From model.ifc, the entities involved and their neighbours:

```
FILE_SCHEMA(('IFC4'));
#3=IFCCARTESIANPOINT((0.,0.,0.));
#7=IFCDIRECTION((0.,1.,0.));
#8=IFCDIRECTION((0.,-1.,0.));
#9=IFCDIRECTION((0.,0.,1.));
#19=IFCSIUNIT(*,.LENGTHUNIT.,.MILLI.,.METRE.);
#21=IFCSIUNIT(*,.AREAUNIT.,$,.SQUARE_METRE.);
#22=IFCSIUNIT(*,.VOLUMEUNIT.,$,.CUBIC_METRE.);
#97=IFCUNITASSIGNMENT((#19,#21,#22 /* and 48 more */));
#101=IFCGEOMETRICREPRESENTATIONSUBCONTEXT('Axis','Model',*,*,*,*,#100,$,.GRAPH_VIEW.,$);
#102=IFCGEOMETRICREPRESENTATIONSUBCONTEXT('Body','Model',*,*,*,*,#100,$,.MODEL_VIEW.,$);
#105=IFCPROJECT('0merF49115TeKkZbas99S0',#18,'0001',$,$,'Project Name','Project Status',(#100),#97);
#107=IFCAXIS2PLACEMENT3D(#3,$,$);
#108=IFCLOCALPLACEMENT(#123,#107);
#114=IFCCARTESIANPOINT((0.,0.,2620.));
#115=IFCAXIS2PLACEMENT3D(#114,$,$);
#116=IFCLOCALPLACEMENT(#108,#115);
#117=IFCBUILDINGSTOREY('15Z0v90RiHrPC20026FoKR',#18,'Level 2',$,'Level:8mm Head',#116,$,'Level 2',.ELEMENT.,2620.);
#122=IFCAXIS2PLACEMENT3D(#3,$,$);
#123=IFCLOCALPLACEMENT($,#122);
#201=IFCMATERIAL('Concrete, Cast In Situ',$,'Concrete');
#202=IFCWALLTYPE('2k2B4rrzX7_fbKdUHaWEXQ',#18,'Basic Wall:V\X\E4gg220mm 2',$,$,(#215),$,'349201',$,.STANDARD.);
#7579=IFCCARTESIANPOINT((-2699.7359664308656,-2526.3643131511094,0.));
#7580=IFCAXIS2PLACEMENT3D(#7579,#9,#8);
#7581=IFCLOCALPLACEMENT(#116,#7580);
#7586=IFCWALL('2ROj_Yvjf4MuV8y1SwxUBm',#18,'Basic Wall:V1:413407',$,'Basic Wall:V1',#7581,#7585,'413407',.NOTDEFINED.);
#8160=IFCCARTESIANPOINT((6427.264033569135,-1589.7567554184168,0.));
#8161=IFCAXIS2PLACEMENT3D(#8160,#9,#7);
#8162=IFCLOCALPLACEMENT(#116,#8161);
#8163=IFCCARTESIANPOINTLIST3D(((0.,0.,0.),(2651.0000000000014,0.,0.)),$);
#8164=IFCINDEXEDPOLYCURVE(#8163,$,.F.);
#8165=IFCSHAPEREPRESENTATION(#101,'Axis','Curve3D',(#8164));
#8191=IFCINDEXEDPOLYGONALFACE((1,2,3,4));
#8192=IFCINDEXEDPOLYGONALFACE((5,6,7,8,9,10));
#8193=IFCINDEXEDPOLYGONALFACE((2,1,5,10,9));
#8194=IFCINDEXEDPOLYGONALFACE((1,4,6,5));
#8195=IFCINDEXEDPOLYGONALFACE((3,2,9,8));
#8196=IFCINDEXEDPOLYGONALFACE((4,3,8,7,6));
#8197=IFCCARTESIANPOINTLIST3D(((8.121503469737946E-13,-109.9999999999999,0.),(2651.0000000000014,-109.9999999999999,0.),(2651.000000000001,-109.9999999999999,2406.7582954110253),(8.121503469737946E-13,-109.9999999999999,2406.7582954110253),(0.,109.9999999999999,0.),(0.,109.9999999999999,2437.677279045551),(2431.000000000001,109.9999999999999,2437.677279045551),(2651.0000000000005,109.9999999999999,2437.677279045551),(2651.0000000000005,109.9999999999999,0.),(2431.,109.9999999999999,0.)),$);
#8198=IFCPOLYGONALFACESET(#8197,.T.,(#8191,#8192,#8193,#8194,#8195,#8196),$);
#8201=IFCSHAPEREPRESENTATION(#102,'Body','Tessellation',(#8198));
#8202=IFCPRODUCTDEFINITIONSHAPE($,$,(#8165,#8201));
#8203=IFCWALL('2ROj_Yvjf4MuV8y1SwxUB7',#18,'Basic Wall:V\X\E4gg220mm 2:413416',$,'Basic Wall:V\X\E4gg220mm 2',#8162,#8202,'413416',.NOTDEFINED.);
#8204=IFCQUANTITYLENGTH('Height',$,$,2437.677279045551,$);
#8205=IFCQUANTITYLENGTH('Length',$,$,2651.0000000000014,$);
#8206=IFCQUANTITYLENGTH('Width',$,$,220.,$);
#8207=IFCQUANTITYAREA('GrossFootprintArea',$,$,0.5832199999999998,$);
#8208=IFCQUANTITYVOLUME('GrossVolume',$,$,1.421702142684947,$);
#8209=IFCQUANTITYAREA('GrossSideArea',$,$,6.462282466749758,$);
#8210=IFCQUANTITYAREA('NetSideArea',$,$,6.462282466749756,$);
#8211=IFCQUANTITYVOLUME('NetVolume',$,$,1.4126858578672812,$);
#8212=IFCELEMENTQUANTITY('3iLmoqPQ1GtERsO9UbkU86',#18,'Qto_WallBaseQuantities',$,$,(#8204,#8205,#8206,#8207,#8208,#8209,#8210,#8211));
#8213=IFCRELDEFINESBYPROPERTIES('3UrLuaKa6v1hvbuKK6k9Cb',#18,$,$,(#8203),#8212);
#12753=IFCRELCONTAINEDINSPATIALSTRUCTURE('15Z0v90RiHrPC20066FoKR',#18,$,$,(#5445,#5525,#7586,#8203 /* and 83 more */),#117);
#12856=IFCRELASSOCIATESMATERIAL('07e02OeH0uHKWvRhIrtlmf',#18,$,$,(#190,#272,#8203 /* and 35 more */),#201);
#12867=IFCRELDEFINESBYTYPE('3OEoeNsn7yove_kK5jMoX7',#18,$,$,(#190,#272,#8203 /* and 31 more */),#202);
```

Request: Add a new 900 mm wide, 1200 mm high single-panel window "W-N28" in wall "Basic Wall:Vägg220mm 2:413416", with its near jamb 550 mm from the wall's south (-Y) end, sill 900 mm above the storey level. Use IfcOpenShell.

```python
import numpy as np
import ifcopenshell
import ifcopenshell.api.feature
import ifcopenshell.api.geometry
import ifcopenshell.api.pset
import ifcopenshell.api.root
import ifcopenshell.api.spatial
import ifcopenshell.geom
import ifcopenshell.util.element
import ifcopenshell.util.placement
import ifcopenshell.util.representation
import ifcopenshell.util.shape
import ifcopenshell.util.unit

model = ifcopenshell.open("model.ifc")
unit_scale = ifcopenshell.util.unit.calculate_unit_scale(model)
area_scale = ifcopenshell.util.unit.calculate_unit_scale(model, "AREAUNIT")
volume_scale = ifcopenshell.util.unit.calculate_unit_scale(model, "VOLUMEUNIT")
settings = ifcopenshell.geom.settings()


def volume(element):
    """Net volume in cubic metres, openings subtracted."""
    shape = ifcopenshell.geom.create_shape(settings, element)
    return ifcopenshell.util.shape.get_volume(shape.geometry)


wall = model.by_guid("2ROj_Yvjf4MuV8y1SwxUB7")
storey = ifcopenshell.util.element.get_container(wall, ifc_class="IfcBuildingStorey")
context = ifcopenshell.util.representation.get_context(model, "Model", "Body", "MODEL_VIEW")
before = volume(wall)

width, height, from_end, sill = 0.9, 1.2, 0.55, 0.9  # metres

# The wall runs along its own X axis, and the end named is its -X end.
wall_shape = ifcopenshell.geom.create_shape(settings, wall)
x, y, z = ifcopenshell.util.shape.get_vertices(wall_shape.geometry).T
start = x.min() + from_end
face, thickness = float(y.min()), float(y.max() - y.min())
wall_matrix = ifcopenshell.util.placement.get_local_placement(wall.ObjectPlacement)
level = ifcopenshell.util.placement.get_local_placement(storey.ObjectPlacement)[2, 3]


def in_wall(x, y):
    """Placement at x, y metres in the wall's axes, at sill height."""
    matrix = wall_matrix.copy()
    matrix[:, 3] = wall_matrix @ np.array([x / unit_scale, y / unit_scale, 0.0, 1.0])
    matrix[2, 3] = level + sill / unit_scale
    return matrix


# Opening: a box that overshoots both wall faces by 50 mm.
opening = ifcopenshell.api.root.create_entity(model, ifc_class="IfcOpeningElement", predefined_type="OPENING")
box = ifcopenshell.api.geometry.add_wall_representation(
    model, context=context, length=width, height=height, thickness=thickness + 0.1
)
ifcopenshell.api.geometry.assign_representation(model, product=opening, representation=box)
ifcopenshell.api.geometry.edit_object_placement(model, product=opening, matrix=in_wall(start, face - 0.05), is_si=False)
ifcopenshell.api.feature.add_feature(model, feature=opening, element=wall)

window = ifcopenshell.api.root.create_entity(model, ifc_class="IfcWindow", name="W-N28", predefined_type="WINDOW")
window.OverallWidth, window.OverallHeight = width / unit_scale, height / unit_scale
window.PartitioningType = "SINGLE_PANEL"
body = ifcopenshell.api.geometry.add_window_representation(
    model,
    context=context,
    overall_width=window.OverallWidth,
    overall_height=window.OverallHeight,
    partition_type="SINGLE_PANEL",
)
ifcopenshell.api.geometry.assign_representation(model, product=window, representation=body)
ifcopenshell.api.spatial.assign_container(model, products=[window], relating_structure=storey)
ifcopenshell.api.feature.add_filling(model, opening=opening, element=window)

# Centre the window in the wall's thickness.
ifcopenshell.api.geometry.edit_object_placement(model, product=window, matrix=in_wall(start, face), is_si=False)
window_shape = ifcopenshell.geom.create_shape(settings, window)
depth = ifcopenshell.util.shape.get_vertices(window_shape.geometry)[:, 1]
offset = face + thickness / 2 - (depth.min() + depth.max()) / 2
ifcopenshell.api.geometry.edit_object_placement(model, product=window, matrix=in_wall(start, offset), is_si=False)

after = volume(wall)

# Update the wall's stored quantities.
qto = model.by_id(ifcopenshell.util.element.get_pset(wall, "Qto_WallBaseQuantities", should_inherit=False)["id"])
ifcopenshell.api.pset.edit_qto(model, qto=qto, properties={
    "NetSideArea": after / thickness / area_scale,
    "NetVolume": after / volume_scale,
})

print(f"wall volume {before:.3f} -> {after:.3f} m3")

model.write("model_edited.ifc")
```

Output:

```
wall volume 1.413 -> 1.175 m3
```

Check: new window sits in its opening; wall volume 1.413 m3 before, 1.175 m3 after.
